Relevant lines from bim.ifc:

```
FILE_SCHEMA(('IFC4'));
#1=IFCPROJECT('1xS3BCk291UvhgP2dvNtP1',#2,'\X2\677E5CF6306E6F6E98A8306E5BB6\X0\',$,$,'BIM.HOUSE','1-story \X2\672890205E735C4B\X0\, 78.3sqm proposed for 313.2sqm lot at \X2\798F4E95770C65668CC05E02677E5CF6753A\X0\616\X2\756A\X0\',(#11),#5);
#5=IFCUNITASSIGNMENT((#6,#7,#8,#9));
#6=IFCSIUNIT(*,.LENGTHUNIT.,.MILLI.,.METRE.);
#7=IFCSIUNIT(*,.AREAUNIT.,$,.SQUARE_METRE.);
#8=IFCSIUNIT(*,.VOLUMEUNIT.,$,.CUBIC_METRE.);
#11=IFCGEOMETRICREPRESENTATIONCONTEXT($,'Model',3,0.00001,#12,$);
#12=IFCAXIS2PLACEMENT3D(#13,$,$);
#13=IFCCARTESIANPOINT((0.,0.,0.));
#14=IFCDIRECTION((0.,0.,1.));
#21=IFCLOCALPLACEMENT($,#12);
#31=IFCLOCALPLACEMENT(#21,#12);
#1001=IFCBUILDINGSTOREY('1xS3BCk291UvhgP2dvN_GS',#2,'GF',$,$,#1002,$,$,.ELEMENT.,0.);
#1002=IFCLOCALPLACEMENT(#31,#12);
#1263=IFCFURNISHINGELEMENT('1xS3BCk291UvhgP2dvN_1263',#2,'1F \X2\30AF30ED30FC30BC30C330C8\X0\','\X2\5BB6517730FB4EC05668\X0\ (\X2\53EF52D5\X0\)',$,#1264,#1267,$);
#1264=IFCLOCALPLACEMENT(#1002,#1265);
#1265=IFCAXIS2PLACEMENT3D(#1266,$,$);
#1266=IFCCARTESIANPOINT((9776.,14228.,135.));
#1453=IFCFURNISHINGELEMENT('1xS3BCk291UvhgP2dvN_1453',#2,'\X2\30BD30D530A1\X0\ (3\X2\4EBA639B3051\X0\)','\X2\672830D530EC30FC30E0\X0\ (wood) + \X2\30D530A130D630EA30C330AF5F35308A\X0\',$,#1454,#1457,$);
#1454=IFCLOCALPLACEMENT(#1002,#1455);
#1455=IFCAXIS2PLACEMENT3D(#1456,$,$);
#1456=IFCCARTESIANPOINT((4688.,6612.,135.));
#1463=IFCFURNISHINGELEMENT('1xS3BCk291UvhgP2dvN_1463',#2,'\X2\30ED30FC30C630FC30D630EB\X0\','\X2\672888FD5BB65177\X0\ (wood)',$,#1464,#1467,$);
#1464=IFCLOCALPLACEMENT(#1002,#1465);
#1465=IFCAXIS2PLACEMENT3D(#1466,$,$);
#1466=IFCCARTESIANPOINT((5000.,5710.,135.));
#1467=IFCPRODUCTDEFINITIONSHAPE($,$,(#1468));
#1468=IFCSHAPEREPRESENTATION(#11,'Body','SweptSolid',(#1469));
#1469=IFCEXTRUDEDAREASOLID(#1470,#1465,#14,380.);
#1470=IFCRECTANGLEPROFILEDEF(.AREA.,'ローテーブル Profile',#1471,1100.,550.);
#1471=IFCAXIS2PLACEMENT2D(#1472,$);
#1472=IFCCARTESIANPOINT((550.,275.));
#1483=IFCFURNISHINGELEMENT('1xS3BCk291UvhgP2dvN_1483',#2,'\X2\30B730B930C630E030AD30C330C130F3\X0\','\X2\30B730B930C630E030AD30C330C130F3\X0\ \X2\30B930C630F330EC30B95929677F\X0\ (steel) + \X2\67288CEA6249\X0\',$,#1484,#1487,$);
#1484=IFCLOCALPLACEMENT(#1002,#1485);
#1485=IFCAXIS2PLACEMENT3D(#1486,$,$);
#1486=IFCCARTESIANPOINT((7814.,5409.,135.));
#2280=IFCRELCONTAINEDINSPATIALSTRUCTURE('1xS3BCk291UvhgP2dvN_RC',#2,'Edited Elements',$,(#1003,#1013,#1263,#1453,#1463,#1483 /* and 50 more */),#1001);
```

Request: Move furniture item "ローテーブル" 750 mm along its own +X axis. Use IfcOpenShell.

```python
import ifcopenshell
import ifcopenshell.api.geometry
import ifcopenshell.util.placement
import ifcopenshell.util.unit

model = ifcopenshell.open("bim.ifc")
unit_scale = ifcopenshell.util.unit.calculate_unit_scale(model)

item = model.by_guid("1xS3BCk291UvhgP2dvN_1463")
matrix = ifcopenshell.util.placement.get_local_placement(item.ObjectPlacement)
matrix[:3, 3] += matrix[:3, 0] * 0.75 / unit_scale
ifcopenshell.api.geometry.edit_object_placement(model, product=item, matrix=matrix, is_si=False)

print(ifcopenshell.util.placement.get_local_placement(item.ObjectPlacement).round(3) + 0.0)

model.write("bim_edited.ifc")
```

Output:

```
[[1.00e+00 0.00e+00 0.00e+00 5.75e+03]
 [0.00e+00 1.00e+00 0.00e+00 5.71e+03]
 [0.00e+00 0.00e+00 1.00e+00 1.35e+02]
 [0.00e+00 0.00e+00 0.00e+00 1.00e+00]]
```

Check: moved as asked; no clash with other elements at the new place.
